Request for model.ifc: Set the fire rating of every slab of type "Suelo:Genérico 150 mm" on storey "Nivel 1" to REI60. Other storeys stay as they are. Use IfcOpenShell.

First a look at what the model holds.

```python
import ifcopenshell
import ifcopenshell.util.element

model = ifcopenshell.open("model.ifc")
print(model.schema)
storey = next(s for s in model.by_type("IfcBuildingStorey") if s.Name == "Nivel 1")
slabs = [e for e in ifcopenshell.util.element.get_decomposition(storey) if e.is_a("IfcSlab")]
seen = {}
for e in slabs:
    element_type = ifcopenshell.util.element.get_type(e)
    key = (element_type.Name if element_type != e and element_type else None, ifcopenshell.util.element.get_pset(e, "Pset_SlabCommon", "FireRating"))
    seen[key] = seen.get(key, 0) + 1
for (name, value), count in sorted(seen.items(), key=str):
    print(count, "x", name, "|", value)
```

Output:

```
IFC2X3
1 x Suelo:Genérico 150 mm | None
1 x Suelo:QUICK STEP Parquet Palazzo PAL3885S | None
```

```python
import ifcopenshell
import ifcopenshell.api.pset
import ifcopenshell.util.element

model = ifcopenshell.open("model.ifc")

storey = next(s for s in model.by_type("IfcBuildingStorey") if s.Name == "Nivel 1")
slabs = [e for e in ifcopenshell.util.element.get_decomposition(storey) if e.is_a("IfcSlab")]

count = 0
for e in slabs:
    element_type = ifcopenshell.util.element.get_type(e)
    if element_type in (None, e) or element_type.Name != "Suelo:Genérico 150 mm":
        continue
    # add_pset returns the element's existing set when there is one.
    pset = ifcopenshell.api.pset.add_pset(model, product=e, name="Pset_SlabCommon")
    ifcopenshell.api.pset.edit_pset(model, pset=pset, properties={"FireRating": "REI60"})
    count += 1

print(count, "slabs updated")

model.write("model_updated.ifc")
```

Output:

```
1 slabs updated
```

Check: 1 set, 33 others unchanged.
